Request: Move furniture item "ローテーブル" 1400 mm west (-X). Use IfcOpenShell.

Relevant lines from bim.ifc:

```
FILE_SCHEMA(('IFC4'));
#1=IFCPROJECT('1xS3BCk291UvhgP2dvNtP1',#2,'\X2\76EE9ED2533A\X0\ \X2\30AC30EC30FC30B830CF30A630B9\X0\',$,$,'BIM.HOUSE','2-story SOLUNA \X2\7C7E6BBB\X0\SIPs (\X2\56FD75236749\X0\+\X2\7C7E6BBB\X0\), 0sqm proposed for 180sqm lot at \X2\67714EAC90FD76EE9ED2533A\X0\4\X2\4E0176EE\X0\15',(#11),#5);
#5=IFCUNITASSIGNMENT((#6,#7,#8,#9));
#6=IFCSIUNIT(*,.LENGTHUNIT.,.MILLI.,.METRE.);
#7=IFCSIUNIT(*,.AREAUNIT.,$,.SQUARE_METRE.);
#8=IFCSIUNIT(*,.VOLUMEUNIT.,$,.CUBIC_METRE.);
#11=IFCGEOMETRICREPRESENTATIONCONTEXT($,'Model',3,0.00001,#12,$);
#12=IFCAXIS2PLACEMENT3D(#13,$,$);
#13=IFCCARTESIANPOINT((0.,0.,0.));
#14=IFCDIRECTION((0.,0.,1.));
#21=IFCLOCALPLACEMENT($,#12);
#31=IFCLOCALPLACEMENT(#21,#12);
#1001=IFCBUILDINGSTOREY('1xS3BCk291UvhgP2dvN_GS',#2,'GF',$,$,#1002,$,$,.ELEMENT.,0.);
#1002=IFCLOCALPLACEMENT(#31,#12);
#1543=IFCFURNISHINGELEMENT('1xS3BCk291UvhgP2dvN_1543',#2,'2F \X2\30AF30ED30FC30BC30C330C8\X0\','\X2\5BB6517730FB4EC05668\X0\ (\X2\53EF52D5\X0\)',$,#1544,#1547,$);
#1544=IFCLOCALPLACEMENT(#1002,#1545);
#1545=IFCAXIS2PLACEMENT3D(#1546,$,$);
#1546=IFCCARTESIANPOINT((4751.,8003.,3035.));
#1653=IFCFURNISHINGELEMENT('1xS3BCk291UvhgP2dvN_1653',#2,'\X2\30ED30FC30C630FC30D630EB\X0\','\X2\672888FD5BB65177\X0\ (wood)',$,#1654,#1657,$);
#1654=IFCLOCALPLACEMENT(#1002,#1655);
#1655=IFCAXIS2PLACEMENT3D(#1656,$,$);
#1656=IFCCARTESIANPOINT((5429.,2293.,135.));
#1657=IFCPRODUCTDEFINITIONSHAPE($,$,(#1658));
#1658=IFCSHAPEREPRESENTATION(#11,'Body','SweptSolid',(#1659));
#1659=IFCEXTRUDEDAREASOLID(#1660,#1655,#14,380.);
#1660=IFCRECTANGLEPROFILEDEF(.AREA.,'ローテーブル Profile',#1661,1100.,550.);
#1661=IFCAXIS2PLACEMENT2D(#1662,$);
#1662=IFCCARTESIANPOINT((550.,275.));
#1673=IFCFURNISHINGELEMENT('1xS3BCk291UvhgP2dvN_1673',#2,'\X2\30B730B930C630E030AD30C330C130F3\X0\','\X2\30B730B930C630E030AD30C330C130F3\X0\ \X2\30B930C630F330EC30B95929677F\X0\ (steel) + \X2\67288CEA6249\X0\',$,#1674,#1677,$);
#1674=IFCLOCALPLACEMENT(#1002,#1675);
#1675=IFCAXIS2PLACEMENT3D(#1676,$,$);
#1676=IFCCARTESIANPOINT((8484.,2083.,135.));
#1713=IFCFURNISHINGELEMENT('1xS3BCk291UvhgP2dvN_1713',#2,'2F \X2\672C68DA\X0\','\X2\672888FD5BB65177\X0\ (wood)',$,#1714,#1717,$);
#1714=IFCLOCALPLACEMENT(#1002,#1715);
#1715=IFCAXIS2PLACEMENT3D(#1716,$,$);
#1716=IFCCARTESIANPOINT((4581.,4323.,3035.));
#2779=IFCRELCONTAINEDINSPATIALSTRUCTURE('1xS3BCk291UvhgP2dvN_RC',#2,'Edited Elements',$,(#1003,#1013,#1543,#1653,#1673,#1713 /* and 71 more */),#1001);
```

```python
import ifcopenshell
import ifcopenshell.api.geometry
import ifcopenshell.util.placement

model = ifcopenshell.open("bim.ifc")

item = model.by_guid("1xS3BCk291UvhgP2dvN_1653")
matrix = ifcopenshell.util.placement.get_local_placement(item.ObjectPlacement)
matrix[0, 3] -= 1400.0
ifcopenshell.api.geometry.edit_object_placement(model, product=item, matrix=matrix, is_si=False)

print(ifcopenshell.util.placement.get_local_placement(item.ObjectPlacement).round(3) + 0.0)

model.write("bim_updated.ifc")
```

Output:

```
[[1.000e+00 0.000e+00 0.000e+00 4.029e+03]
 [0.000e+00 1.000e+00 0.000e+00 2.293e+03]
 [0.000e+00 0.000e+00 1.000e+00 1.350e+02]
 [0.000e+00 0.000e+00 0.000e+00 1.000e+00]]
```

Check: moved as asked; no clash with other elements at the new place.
